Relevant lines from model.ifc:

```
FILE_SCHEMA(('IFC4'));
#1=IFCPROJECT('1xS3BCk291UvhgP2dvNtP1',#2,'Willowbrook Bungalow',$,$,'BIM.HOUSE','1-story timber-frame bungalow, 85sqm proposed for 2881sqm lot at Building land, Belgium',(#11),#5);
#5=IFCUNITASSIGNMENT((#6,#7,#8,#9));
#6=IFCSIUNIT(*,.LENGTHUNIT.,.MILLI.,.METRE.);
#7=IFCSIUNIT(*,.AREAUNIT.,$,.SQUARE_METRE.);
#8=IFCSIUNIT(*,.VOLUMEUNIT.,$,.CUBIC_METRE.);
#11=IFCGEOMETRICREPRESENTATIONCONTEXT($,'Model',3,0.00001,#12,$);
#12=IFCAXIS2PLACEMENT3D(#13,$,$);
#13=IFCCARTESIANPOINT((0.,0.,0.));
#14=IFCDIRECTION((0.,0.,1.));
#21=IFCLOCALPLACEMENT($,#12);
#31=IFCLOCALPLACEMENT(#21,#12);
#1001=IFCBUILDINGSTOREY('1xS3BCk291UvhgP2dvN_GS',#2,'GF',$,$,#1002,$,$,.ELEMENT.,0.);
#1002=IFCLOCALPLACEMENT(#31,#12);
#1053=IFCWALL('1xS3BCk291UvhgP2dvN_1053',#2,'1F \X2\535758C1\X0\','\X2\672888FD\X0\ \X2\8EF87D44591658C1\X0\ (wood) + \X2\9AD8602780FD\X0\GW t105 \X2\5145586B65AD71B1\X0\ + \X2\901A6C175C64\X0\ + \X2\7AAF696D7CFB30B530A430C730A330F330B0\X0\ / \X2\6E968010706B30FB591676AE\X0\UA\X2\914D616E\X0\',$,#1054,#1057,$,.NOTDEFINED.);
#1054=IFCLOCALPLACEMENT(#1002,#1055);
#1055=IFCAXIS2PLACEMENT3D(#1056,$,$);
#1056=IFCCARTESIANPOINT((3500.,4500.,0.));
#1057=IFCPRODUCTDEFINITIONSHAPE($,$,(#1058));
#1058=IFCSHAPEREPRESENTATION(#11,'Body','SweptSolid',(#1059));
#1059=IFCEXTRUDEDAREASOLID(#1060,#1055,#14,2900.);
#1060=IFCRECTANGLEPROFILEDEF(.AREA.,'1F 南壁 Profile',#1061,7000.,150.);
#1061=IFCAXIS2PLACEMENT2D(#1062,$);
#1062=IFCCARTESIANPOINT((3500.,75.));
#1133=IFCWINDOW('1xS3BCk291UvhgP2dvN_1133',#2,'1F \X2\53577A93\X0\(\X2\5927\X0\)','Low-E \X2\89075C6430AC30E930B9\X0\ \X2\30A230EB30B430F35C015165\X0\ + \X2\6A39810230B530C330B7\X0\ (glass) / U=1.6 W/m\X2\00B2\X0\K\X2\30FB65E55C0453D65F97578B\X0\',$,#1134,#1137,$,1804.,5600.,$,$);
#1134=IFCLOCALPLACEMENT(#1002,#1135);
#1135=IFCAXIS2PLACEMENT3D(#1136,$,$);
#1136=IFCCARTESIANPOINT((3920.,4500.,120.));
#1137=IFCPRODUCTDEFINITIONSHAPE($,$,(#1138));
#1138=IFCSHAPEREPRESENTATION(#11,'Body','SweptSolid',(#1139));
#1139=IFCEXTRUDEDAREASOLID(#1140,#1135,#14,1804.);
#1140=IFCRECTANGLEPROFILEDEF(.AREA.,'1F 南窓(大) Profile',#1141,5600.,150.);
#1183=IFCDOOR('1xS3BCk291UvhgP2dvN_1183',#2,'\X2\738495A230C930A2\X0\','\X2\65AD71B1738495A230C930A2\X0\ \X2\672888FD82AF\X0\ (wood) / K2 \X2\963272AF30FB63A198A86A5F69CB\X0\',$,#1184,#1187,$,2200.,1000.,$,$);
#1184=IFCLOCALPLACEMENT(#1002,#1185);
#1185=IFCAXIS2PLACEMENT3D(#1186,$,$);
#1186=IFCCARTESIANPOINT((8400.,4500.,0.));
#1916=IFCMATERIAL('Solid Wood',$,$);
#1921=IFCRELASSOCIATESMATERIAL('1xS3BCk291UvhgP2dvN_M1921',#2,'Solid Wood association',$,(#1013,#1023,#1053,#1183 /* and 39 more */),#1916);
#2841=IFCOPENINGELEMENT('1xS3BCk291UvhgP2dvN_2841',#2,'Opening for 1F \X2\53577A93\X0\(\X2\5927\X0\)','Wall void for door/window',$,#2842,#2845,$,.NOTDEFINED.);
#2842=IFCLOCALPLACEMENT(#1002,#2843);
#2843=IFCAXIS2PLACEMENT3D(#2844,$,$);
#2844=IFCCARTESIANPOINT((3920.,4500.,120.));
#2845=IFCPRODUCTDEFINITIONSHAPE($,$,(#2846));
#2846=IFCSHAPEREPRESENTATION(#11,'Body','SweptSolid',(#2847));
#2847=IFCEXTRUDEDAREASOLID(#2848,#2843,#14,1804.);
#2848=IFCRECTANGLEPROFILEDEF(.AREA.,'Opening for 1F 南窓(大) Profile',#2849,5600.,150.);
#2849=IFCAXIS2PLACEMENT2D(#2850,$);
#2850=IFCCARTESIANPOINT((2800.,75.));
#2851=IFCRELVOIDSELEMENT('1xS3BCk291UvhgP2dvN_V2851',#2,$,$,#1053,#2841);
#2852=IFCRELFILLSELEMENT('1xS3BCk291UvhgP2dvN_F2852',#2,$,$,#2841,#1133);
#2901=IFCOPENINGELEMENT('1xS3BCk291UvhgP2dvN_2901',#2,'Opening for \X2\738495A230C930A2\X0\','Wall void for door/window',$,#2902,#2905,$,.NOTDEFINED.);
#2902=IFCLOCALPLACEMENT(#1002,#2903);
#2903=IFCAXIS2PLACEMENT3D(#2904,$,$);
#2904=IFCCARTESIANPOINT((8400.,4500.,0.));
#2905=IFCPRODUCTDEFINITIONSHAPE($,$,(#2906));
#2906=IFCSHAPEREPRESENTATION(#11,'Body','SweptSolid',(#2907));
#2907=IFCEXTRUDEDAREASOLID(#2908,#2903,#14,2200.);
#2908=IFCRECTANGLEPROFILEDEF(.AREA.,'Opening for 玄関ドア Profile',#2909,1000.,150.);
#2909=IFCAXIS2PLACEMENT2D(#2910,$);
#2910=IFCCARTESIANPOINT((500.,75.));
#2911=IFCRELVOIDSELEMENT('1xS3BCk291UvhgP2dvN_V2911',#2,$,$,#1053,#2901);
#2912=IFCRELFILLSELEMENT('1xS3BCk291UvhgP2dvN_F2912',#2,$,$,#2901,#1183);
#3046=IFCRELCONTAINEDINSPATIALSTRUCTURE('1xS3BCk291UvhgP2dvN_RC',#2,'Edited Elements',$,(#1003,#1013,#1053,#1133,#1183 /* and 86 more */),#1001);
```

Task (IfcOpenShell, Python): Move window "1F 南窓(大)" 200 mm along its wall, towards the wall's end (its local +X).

```python
import ifcopenshell
import ifcopenshell.api.geometry
import ifcopenshell.util.placement

model = ifcopenshell.open("model.ifc")

window = model.by_guid("1xS3BCk291UvhgP2dvN_1133")
opening = window.FillsVoids[0].RelatingOpeningElement
wall = opening.VoidsElements[0].RelatingBuildingElement

wall_matrix = ifcopenshell.util.placement.get_local_placement(wall.ObjectPlacement)
shift = wall_matrix[:3, 0] * 200.0
before = ifcopenshell.util.placement.get_local_placement(window.ObjectPlacement)[:3, 3].copy()

# The window is not placed relative to its opening, so move both.
for product in (opening, window):
    matrix = ifcopenshell.util.placement.get_local_placement(product.ObjectPlacement)
    matrix[:3, 3] += shift
    ifcopenshell.api.geometry.edit_object_placement(model, product=product, matrix=matrix, is_si=False)

after = ifcopenshell.util.placement.get_local_placement(window.ObjectPlacement)[:3, 3]
print("window moved by", (after - before).round(3) + 0.0)

model.write("model_edited.ifc")
```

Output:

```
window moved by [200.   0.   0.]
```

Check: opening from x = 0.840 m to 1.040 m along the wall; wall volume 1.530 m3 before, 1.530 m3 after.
